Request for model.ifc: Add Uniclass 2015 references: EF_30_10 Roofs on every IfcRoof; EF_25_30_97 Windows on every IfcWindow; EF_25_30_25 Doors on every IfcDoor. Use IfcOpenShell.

First a look at what the model holds.

```python
import ifcopenshell

model = ifcopenshell.open("model.ifc")
print(model.schema)
print("classifications:", [c.Name for c in model.by_type("IfcClassification")])
for ifc_class in ("IfcDoor", "IfcRoof", "IfcStair", "IfcWall", "IfcWindow"):
    print(ifc_class, len(model.by_type(ifc_class)))
```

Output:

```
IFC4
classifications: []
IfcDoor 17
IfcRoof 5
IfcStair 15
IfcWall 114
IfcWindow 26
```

```python
import ifcopenshell
import ifcopenshell.api.classification

model = ifcopenshell.open("model.ifc")

system = ifcopenshell.api.classification.add_classification(model, classification="Uniclass 2015")

codes = {
    "IfcRoof": ("EF_30_10", "Roofs"),
    "IfcWindow": ("EF_25_30_97", "Windows"),
    "IfcDoor": ("EF_25_30_25", "Doors"),
}
for ifc_class, (code, name) in codes.items():
    products = model.by_type(ifc_class)
    ifcopenshell.api.classification.add_reference(
        model, products=products, classification=system, identification=code, name=name
    )
    print(code, len(products))

model.write("model-out.ifc")
```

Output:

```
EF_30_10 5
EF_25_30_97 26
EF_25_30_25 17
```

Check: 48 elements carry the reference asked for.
